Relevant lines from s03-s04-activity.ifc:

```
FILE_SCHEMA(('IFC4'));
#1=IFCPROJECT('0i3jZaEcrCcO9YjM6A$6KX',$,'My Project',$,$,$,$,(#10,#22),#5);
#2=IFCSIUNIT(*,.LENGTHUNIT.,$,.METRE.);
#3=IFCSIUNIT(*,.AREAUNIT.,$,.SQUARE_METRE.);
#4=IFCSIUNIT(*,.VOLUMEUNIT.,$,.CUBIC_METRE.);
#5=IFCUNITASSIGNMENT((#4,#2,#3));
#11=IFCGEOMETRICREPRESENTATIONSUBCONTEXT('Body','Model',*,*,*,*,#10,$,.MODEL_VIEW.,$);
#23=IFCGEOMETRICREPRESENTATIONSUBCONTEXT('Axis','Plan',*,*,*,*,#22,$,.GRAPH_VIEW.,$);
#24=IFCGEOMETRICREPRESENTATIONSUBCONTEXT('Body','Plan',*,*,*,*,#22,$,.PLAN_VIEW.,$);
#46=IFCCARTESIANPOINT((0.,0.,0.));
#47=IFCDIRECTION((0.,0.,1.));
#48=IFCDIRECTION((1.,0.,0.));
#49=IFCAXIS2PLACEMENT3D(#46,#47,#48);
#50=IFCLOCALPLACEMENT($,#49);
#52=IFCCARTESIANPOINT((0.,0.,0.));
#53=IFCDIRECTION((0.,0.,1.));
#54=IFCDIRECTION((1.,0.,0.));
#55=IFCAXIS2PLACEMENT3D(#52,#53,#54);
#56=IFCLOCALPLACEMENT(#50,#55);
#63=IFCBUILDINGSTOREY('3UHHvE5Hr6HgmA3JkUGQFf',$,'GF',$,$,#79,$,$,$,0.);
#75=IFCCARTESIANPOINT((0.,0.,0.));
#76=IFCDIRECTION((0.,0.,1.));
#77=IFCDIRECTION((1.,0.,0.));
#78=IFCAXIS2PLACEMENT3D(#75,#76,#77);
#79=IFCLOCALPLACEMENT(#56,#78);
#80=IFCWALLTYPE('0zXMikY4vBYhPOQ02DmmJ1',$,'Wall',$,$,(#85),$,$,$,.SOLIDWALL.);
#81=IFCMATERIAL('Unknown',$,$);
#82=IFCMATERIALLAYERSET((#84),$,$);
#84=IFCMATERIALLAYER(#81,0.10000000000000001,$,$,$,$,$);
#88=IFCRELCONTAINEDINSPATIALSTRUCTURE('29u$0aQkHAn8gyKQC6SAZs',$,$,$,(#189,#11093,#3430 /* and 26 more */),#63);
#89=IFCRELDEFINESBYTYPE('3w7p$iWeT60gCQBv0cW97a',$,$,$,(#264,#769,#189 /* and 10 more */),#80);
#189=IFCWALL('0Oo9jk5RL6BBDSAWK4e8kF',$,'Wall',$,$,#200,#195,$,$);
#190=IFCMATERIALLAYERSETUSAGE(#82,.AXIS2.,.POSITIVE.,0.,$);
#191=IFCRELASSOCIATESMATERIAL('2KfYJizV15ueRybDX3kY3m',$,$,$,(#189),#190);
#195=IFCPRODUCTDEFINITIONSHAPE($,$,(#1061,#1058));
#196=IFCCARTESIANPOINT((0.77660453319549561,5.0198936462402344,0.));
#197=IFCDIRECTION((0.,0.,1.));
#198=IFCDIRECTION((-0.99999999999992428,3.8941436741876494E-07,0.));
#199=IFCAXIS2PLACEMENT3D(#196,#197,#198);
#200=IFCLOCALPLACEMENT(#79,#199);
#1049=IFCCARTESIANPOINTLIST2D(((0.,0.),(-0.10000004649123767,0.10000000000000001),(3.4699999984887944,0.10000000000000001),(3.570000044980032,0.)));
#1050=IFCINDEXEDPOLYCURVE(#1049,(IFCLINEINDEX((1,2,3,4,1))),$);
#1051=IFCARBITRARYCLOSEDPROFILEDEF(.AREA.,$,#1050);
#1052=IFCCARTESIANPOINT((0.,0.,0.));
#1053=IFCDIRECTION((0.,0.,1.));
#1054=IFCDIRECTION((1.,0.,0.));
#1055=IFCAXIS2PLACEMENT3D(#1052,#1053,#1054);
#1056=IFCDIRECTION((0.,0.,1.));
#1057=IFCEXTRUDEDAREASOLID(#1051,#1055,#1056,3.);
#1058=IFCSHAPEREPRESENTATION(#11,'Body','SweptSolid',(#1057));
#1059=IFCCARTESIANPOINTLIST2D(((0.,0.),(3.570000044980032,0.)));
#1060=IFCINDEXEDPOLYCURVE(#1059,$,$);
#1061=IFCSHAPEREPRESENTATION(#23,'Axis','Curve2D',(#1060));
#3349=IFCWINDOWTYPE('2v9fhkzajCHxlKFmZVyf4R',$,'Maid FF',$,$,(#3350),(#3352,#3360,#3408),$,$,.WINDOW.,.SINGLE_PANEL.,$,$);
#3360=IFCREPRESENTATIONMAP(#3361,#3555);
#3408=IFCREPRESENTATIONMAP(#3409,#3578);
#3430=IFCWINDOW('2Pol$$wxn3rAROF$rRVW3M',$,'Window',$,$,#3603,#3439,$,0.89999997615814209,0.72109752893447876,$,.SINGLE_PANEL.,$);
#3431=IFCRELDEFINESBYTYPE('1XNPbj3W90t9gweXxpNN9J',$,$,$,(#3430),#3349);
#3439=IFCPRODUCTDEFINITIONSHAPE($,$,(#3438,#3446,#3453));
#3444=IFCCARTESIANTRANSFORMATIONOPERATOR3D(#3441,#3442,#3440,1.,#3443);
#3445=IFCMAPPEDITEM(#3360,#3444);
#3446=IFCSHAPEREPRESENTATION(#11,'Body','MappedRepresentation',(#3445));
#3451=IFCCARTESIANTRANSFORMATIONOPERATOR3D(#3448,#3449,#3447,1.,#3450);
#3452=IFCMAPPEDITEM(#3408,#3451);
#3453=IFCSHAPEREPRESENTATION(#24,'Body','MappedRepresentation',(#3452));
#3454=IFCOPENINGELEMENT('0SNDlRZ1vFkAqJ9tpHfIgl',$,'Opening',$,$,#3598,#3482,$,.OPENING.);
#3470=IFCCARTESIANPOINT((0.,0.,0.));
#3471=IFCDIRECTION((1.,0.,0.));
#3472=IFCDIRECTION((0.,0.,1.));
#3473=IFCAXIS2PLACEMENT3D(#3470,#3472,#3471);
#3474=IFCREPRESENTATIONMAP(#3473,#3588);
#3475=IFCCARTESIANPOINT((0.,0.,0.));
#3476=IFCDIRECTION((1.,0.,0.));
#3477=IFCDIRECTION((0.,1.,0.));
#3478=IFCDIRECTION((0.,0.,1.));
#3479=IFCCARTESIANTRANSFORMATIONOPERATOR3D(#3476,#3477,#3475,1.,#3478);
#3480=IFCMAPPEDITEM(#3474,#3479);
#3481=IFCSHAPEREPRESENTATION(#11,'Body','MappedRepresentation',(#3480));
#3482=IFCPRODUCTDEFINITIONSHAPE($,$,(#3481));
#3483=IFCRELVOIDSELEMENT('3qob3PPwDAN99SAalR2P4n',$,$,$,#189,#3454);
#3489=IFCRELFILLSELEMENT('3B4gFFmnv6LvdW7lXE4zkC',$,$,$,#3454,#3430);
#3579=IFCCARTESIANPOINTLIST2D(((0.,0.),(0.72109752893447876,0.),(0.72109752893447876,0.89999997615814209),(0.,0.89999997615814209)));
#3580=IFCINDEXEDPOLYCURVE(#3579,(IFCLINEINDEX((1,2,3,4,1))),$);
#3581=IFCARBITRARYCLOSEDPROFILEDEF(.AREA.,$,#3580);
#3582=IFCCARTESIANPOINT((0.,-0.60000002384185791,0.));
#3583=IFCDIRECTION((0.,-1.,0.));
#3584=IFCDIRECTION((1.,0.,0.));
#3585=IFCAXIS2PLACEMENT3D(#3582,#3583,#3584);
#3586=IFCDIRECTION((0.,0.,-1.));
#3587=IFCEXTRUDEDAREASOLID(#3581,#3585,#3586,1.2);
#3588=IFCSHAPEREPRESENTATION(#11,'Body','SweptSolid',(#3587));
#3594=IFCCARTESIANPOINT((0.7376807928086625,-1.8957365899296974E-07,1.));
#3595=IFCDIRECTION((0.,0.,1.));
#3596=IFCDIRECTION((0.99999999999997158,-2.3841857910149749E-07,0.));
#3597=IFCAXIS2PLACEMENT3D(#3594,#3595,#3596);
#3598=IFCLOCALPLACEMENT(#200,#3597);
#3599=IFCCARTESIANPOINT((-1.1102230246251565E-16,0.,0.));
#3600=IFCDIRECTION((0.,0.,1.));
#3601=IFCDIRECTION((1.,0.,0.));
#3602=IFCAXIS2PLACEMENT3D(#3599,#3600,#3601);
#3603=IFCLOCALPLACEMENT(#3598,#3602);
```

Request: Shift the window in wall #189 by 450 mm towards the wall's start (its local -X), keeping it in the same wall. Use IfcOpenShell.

```python
import ifcopenshell
import ifcopenshell.api.geometry
import ifcopenshell.util.placement

model = ifcopenshell.open("s03-s04-activity.ifc")

window = model.by_id(3430)
opening = window.FillsVoids[0].RelatingOpeningElement
wall = opening.VoidsElements[0].RelatingBuildingElement

wall_matrix = ifcopenshell.util.placement.get_local_placement(wall.ObjectPlacement)
shift = wall_matrix[:3, 0] * -0.45
before = ifcopenshell.util.placement.get_local_placement(window.ObjectPlacement)[:3, 3].copy()

# The window is placed relative to its opening, so it follows when the opening moves.
matrix = ifcopenshell.util.placement.get_local_placement(opening.ObjectPlacement)
matrix[:3, 3] += shift
ifcopenshell.api.geometry.edit_object_placement(
    model, product=opening, matrix=matrix, is_si=False, should_transform_children=True
)

after = ifcopenshell.util.placement.get_local_placement(window.ObjectPlacement)[:3, 3]
print("window moved by", (after - before).round(3) + 0.0)

model.write("s03-s04-activity_updated.ifc")
```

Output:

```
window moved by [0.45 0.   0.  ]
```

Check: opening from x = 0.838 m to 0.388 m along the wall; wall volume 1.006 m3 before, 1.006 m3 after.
